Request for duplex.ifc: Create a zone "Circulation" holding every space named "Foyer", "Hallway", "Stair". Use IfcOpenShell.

First a look at what the model holds.

```python
import ifcopenshell

model = ifcopenshell.open("duplex.ifc")
print(model.schema)
seen = {}
for space in model.by_type("IfcSpace"):
    seen[space.LongName] = seen.get(space.LongName, 0) + 1
for name, count in sorted(seen.items(), key=str):
    print(count, "x", name)
print("zones:", [z.Name for z in model.by_type("IfcZone")][:20])
```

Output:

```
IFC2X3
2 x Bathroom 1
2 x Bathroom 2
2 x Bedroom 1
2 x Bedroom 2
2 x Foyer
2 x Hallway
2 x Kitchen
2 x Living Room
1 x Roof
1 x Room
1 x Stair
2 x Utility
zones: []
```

```python
import ifcopenshell
import ifcopenshell.api.group
import ifcopenshell.api.root

model = ifcopenshell.open("duplex.ifc")

names = {"Foyer", "Hallway", "Stair"}
spaces = [s for s in model.by_type("IfcSpace") if s.LongName in names]

zone = ifcopenshell.api.root.create_entity(model, ifc_class="IfcZone", name="Circulation")
ifcopenshell.api.group.assign_group(model, products=spaces, group=zone)
print(len(spaces), "spaces in", zone.Name)

model.write("duplex_rev.ifc")
```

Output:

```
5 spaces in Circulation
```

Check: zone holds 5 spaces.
